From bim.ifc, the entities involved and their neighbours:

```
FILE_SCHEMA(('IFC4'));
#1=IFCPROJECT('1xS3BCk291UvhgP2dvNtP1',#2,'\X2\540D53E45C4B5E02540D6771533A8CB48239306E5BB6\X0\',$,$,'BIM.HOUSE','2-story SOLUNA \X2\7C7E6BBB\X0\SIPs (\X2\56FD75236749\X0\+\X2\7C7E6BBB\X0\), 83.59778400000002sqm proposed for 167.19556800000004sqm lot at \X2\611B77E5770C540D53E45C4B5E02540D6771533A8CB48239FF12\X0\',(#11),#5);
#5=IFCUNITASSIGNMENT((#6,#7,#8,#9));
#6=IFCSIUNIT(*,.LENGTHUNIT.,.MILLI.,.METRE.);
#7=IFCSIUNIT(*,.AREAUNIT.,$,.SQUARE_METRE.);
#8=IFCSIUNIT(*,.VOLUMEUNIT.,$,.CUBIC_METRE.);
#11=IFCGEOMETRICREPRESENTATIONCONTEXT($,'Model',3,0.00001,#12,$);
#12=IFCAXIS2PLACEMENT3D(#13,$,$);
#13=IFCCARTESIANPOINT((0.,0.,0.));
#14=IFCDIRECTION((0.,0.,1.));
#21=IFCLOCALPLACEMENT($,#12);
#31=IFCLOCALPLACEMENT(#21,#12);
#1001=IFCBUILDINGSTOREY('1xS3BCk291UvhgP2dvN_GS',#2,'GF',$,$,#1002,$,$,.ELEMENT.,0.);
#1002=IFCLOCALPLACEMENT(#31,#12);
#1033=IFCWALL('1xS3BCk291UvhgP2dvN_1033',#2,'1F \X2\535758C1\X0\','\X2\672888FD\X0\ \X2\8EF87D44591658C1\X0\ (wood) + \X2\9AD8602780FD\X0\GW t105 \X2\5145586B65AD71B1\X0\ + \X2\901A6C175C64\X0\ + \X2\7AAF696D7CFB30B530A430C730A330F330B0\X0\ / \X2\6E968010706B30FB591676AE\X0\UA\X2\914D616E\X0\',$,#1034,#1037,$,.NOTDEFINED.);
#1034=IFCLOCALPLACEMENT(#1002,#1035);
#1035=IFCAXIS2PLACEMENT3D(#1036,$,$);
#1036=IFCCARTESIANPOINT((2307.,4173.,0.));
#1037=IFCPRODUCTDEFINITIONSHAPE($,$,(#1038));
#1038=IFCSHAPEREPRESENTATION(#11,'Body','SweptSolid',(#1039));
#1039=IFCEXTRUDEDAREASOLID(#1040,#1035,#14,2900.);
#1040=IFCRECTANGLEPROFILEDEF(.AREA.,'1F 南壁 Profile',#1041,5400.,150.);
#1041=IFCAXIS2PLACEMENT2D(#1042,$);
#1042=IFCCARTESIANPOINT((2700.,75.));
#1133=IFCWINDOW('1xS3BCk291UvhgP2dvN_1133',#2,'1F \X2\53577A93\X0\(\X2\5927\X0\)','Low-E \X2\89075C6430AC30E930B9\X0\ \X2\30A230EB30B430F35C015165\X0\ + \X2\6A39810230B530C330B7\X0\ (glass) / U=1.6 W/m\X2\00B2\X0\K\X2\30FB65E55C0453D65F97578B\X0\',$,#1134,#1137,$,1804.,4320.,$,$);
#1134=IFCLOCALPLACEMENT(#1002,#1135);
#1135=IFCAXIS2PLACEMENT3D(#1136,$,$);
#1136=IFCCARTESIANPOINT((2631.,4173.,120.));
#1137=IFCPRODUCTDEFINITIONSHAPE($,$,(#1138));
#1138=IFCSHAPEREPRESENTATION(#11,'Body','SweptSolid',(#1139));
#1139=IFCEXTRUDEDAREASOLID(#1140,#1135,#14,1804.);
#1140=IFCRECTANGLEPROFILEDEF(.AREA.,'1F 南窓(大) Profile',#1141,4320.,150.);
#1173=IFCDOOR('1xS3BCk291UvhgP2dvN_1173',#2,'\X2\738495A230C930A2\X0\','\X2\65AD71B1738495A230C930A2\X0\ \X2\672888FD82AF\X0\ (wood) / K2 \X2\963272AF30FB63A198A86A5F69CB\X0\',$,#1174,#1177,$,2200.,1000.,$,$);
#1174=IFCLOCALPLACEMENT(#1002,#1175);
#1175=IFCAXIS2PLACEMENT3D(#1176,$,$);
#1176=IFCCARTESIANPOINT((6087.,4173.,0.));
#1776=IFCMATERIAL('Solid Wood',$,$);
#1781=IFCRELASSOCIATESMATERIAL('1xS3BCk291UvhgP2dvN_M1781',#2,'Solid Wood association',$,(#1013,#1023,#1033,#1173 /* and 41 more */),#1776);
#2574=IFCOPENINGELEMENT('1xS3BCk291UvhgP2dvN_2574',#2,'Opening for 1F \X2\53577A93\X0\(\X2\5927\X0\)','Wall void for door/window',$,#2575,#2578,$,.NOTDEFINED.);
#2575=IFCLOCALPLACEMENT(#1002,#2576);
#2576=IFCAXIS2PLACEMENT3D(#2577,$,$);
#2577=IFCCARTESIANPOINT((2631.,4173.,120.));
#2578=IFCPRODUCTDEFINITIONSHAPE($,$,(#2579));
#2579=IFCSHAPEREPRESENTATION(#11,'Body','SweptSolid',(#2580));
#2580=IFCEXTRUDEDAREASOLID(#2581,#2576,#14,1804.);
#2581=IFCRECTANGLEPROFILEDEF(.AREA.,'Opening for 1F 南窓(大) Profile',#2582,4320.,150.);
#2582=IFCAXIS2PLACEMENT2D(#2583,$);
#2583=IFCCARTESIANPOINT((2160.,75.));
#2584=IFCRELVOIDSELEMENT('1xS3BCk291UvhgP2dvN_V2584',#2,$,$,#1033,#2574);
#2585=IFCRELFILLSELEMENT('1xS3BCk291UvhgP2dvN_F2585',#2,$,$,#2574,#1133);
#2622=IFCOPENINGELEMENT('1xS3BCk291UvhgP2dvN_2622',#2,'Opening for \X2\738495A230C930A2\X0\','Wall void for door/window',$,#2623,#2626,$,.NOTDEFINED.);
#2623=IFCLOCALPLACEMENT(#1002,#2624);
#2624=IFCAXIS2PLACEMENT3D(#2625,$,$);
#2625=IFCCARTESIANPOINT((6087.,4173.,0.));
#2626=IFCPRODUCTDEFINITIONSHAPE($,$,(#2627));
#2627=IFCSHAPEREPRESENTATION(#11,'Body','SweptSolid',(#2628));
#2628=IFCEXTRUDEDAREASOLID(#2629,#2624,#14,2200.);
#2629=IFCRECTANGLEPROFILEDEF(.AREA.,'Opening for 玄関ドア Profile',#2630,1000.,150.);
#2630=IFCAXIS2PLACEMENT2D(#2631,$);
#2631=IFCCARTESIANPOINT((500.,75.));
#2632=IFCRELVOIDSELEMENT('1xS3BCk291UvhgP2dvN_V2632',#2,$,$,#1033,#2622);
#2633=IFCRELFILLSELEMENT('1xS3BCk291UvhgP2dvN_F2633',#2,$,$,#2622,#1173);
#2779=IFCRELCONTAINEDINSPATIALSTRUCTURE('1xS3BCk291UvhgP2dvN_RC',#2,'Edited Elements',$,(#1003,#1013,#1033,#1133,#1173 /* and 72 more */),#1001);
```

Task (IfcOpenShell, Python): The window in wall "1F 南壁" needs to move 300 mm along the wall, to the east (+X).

```python
import ifcopenshell
import ifcopenshell.api.geometry
import ifcopenshell.util.placement
import ifcopenshell.util.unit

model = ifcopenshell.open("bim.ifc")
unit_scale = ifcopenshell.util.unit.calculate_unit_scale(model)

window = model.by_id(1133)
opening = window.FillsVoids[0].RelatingOpeningElement
wall = opening.VoidsElements[0].RelatingBuildingElement

wall_matrix = ifcopenshell.util.placement.get_local_placement(wall.ObjectPlacement)
shift = wall_matrix[:3, 0] * 0.3 / unit_scale
before = ifcopenshell.util.placement.get_local_placement(window.ObjectPlacement)[:3, 3].copy()

# The window is not placed relative to its opening, so move both.
for product in (opening, window):
    matrix = ifcopenshell.util.placement.get_local_placement(product.ObjectPlacement)
    matrix[:3, 3] += shift
    ifcopenshell.api.geometry.edit_object_placement(model, product=product, matrix=matrix, is_si=False)

after = ifcopenshell.util.placement.get_local_placement(window.ObjectPlacement)[:3, 3]
print("window moved by", (after - before).round(3) + 0.0)

model.write("bim_updated.ifc")
```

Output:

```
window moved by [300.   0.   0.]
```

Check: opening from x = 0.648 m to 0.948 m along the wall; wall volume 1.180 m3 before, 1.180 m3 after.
